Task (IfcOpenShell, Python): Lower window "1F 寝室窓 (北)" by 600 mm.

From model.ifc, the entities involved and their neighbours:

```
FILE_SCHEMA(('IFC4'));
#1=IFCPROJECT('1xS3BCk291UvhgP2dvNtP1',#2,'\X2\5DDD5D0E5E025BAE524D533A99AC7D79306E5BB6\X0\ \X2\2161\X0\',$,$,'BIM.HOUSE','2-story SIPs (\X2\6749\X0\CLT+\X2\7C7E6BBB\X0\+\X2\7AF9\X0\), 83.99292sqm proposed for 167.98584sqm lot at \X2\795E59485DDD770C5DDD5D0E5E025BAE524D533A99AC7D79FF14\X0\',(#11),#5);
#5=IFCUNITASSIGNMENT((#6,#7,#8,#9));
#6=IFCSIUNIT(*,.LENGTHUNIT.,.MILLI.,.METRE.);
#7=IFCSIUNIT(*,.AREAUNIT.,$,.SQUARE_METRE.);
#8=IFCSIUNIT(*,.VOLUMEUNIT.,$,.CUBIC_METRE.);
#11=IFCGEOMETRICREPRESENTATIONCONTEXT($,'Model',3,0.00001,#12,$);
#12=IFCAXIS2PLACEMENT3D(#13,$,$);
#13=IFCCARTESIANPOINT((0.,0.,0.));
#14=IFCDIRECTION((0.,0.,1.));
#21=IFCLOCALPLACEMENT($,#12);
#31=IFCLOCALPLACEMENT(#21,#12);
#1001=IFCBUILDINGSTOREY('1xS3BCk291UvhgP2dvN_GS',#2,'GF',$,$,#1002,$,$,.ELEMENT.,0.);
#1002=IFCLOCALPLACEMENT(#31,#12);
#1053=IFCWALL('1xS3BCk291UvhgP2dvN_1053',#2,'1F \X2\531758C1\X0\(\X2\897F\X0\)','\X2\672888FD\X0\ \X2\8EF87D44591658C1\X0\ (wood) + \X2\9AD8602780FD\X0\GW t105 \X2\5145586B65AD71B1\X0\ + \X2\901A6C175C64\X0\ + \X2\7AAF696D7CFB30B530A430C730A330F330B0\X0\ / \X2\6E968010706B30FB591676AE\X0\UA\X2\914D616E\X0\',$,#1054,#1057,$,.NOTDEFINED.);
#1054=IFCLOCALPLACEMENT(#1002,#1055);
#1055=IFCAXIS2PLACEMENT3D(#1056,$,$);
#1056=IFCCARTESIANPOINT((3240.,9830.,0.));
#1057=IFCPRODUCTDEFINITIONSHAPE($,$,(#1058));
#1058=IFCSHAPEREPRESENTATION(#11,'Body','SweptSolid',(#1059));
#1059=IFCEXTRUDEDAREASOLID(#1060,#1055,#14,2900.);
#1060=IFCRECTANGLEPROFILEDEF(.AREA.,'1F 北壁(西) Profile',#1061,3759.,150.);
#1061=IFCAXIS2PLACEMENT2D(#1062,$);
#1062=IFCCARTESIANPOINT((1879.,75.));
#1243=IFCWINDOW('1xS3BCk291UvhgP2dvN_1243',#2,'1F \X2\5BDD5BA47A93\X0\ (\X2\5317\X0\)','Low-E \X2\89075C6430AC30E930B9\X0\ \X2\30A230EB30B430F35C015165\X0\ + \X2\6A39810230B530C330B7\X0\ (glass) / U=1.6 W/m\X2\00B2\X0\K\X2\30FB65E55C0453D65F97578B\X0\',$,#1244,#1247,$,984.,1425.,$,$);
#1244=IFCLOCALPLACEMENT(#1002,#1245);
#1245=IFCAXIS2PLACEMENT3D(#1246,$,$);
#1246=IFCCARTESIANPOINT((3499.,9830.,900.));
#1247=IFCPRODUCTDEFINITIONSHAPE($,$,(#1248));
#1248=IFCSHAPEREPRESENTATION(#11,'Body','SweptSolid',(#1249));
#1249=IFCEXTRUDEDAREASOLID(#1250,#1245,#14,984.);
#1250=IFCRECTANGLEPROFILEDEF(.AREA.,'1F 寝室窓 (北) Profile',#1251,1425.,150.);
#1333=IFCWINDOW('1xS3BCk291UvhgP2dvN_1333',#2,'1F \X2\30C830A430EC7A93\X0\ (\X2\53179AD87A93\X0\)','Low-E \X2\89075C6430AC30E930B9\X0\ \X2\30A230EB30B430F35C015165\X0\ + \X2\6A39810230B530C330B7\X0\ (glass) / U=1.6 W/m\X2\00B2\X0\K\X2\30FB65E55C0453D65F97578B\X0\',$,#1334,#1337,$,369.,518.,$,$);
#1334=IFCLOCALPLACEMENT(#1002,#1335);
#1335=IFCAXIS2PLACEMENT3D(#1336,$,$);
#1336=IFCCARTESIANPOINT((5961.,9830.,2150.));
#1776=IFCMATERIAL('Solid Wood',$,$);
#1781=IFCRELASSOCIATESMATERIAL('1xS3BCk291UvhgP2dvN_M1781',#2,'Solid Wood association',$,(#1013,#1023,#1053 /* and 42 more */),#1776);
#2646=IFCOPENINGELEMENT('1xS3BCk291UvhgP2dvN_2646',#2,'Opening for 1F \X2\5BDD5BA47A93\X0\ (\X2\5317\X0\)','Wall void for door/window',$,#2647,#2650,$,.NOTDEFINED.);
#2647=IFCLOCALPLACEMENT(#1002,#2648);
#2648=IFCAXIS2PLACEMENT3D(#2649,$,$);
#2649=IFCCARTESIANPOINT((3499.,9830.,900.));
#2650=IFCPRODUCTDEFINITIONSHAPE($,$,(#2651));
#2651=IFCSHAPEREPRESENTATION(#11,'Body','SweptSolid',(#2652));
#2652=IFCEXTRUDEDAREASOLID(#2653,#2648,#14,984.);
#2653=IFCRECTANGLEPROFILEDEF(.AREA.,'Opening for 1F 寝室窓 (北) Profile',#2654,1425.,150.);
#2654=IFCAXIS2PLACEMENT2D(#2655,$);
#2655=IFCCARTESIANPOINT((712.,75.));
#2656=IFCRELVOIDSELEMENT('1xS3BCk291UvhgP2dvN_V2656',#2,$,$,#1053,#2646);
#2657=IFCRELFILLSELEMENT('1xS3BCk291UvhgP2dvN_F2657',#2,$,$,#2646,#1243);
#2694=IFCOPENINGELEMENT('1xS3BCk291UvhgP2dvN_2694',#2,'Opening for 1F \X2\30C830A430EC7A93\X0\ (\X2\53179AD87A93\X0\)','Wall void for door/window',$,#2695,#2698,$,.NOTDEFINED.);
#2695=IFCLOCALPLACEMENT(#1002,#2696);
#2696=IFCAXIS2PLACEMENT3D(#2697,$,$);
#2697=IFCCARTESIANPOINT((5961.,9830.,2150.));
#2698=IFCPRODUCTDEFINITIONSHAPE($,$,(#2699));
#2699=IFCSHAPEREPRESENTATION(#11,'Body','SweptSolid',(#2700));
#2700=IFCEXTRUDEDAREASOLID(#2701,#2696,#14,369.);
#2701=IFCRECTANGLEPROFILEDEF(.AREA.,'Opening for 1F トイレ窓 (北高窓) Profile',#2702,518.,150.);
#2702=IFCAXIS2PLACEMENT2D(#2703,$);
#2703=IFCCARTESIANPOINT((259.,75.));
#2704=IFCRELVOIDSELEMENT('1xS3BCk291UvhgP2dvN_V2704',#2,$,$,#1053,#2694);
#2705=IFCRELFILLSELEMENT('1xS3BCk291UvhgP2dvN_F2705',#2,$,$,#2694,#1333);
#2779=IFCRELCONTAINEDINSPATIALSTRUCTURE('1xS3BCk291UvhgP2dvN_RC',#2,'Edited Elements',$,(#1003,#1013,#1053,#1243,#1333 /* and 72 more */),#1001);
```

```python
import numpy as np
import ifcopenshell
import ifcopenshell.api.geometry
import ifcopenshell.util.placement
import ifcopenshell.util.unit

model = ifcopenshell.open("model.ifc")
unit_scale = ifcopenshell.util.unit.calculate_unit_scale(model)

window = model.by_id(1243)
opening = window.FillsVoids[0].RelatingOpeningElement
dz = -0.6 / unit_scale

shift = np.array([0.0, 0.0, dz])
# The window is not placed relative to its opening, so move both.
for product in (opening, window):
    matrix = ifcopenshell.util.placement.get_local_placement(product.ObjectPlacement)
    matrix[:3, 3] += shift
    ifcopenshell.api.geometry.edit_object_placement(model, product=product, matrix=matrix, is_si=False)

print(f"moved by {dz * unit_scale:+.3f} m")

model.write("model_v2.ifc")
```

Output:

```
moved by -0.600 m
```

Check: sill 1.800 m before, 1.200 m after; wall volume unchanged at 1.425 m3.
